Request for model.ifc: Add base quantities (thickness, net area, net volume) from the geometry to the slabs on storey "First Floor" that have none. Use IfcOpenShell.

First a look at what the model holds.

```python
import ifcopenshell
import ifcopenshell.util.element
import ifcopenshell.util.unit

model = ifcopenshell.open("model.ifc")
print(model.schema)
for unit_type in ("LENGTHUNIT", "AREAUNIT", "VOLUMEUNIT"):
    print(unit_type, ifcopenshell.util.unit.calculate_unit_scale(model, unit_type))
storey = next(s for s in model.by_type("IfcBuildingStorey") if s.Name == "First Floor")
slabs = [e for e in ifcopenshell.util.element.get_decomposition(storey) if e.is_a("IfcSlab")]
for e in sorted(slabs, key=lambda e: e.id()):
    print(e.id(), e.is_a(), e.Name, list(ifcopenshell.util.element.get_psets(e, qtos_only=True)), sep=" | ")
```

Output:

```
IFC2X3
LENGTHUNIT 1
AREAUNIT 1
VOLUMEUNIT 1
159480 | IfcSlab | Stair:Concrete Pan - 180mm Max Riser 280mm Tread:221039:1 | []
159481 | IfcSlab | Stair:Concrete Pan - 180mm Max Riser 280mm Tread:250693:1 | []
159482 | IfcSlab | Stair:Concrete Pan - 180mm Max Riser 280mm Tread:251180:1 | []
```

```python
import ifcopenshell
import ifcopenshell.api.pset
import ifcopenshell.geom
import ifcopenshell.util.element
import ifcopenshell.util.shape
import ifcopenshell.util.unit

model = ifcopenshell.open("model.ifc")
unit_scale = ifcopenshell.util.unit.calculate_unit_scale(model)
area_scale = ifcopenshell.util.unit.calculate_unit_scale(model, "AREAUNIT")
volume_scale = ifcopenshell.util.unit.calculate_unit_scale(model, "VOLUMEUNIT")
settings = ifcopenshell.geom.settings()

storey = next(s for s in model.by_type("IfcBuildingStorey") if s.Name == "First Floor")
slabs = [e for e in ifcopenshell.util.element.get_decomposition(storey) if e.is_a("IfcSlab")]

for e in sorted(slabs, key=lambda e: e.id()):
    if ifcopenshell.util.element.get_psets(e, qtos_only=True, should_inherit=False):
        continue
    # Geometry comes back in metres, in the element's own axes.
    shape = ifcopenshell.geom.create_shape(settings, e)
    values = {
        "Width": ifcopenshell.util.shape.get_z(shape.geometry) / unit_scale,
        "NetArea": ifcopenshell.util.shape.get_footprint_area(shape.geometry) / area_scale,
        "NetVolume": ifcopenshell.util.shape.get_volume(shape.geometry) / volume_scale,
    }
    qto = ifcopenshell.api.pset.add_qto(model, product=e, name="BaseQuantities")
    ifcopenshell.api.pset.edit_qto(model, qto=qto, properties=values)
    print(e.id(), {k: round(v, 3) for k, v in values.items()})

model.write("model_v2.ifc")
```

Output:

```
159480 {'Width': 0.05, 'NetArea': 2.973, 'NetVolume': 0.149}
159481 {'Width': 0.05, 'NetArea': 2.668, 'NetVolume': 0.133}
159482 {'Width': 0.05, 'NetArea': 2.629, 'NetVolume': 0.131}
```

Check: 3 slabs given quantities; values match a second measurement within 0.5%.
